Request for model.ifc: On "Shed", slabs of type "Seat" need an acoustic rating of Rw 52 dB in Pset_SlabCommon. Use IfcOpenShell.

First a look at what the model holds.

```python
import ifcopenshell
import ifcopenshell.util.element

model = ifcopenshell.open("model.ifc")
print(model.schema)
storey = next(s for s in model.by_type("IfcBuildingStorey") if s.Name == "Shed")
slabs = [e for e in ifcopenshell.util.element.get_decomposition(storey) if e.is_a("IfcSlab")]
seen = {}
for e in slabs:
    element_type = ifcopenshell.util.element.get_type(e)
    key = (element_type.Name if element_type != e and element_type else None, ifcopenshell.util.element.get_pset(e, "Pset_SlabCommon", "AcousticRating"))
    seen[key] = seen.get(key, 0) + 1
for (name, value), count in sorted(seen.items(), key=str):
    print(count, "x", name, "|", value)
```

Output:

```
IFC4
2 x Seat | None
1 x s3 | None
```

```python
import ifcopenshell
import ifcopenshell.api.pset
import ifcopenshell.util.element

model = ifcopenshell.open("model.ifc")

storey = next(s for s in model.by_type("IfcBuildingStorey") if s.Name == "Shed")
slabs = [e for e in ifcopenshell.util.element.get_decomposition(storey) if e.is_a("IfcSlab")]

count = 0
for e in slabs:
    element_type = ifcopenshell.util.element.get_type(e)
    if element_type in (None, e) or element_type.Name != "Seat":
        continue
    # add_pset returns the element's existing set when there is one.
    pset = ifcopenshell.api.pset.add_pset(model, product=e, name="Pset_SlabCommon")
    ifcopenshell.api.pset.edit_pset(model, pset=pset, properties={"AcousticRating": "Rw 52 dB"})
    count += 1

print(count, "slabs updated")

model.write("model_rev.ifc")
```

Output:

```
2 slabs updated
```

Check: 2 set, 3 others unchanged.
